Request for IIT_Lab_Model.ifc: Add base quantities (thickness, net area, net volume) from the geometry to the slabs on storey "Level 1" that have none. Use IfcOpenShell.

First a look at what the model holds.

```python
import ifcopenshell
import ifcopenshell.util.element
import ifcopenshell.util.unit

model = ifcopenshell.open("IIT_Lab_Model.ifc")
print(model.schema)
for unit_type in ("LENGTHUNIT", "AREAUNIT", "VOLUMEUNIT"):
    print(unit_type, ifcopenshell.util.unit.calculate_unit_scale(model, unit_type))
storey = next(s for s in model.by_type("IfcBuildingStorey") if s.Name == "Level 1")
slabs = [e for e in ifcopenshell.util.element.get_decomposition(storey) if e.is_a("IfcSlab")]
for e in sorted(slabs, key=lambda e: e.id()):
    print(e.id(), e.is_a(), e.Name, list(ifcopenshell.util.element.get_psets(e, qtos_only=True)), sep=" | ")
```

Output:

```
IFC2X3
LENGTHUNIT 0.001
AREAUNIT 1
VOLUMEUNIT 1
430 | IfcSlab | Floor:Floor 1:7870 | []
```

```python
import ifcopenshell
import ifcopenshell.api.pset
import ifcopenshell.geom
import ifcopenshell.util.element
import ifcopenshell.util.shape
import ifcopenshell.util.unit

model = ifcopenshell.open("IIT_Lab_Model.ifc")
unit_scale = ifcopenshell.util.unit.calculate_unit_scale(model)
area_scale = ifcopenshell.util.unit.calculate_unit_scale(model, "AREAUNIT")
volume_scale = ifcopenshell.util.unit.calculate_unit_scale(model, "VOLUMEUNIT")
settings = ifcopenshell.geom.settings()

storey = next(s for s in model.by_type("IfcBuildingStorey") if s.Name == "Level 1")
slabs = [e for e in ifcopenshell.util.element.get_decomposition(storey) if e.is_a("IfcSlab")]

for e in sorted(slabs, key=lambda e: e.id()):
    if ifcopenshell.util.element.get_psets(e, qtos_only=True, should_inherit=False):
        continue
    # Geometry comes back in metres, in the element's own axes.
    shape = ifcopenshell.geom.create_shape(settings, e)
    values = {
        "Width": ifcopenshell.util.shape.get_z(shape.geometry) / unit_scale,
        "NetArea": ifcopenshell.util.shape.get_footprint_area(shape.geometry) / area_scale,
        "NetVolume": ifcopenshell.util.shape.get_volume(shape.geometry) / volume_scale,
    }
    qto = ifcopenshell.api.pset.add_qto(model, product=e, name="BaseQuantities")
    ifcopenshell.api.pset.edit_qto(model, qto=qto, properties=values)
    print(e.id(), {k: round(v, 3) for k, v in values.items()})

model.write("IIT_Lab_Model_updated.ifc")
```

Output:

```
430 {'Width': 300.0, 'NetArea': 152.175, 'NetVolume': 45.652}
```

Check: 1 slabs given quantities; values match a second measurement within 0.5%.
